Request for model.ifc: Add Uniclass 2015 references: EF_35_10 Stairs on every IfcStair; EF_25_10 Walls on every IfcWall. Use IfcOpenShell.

First a look at what the model holds.

```python
import ifcopenshell

model = ifcopenshell.open("model.ifc")
print(model.schema)
print("classifications:", [c.Name for c in model.by_type("IfcClassification")])
for ifc_class in ("IfcDoor", "IfcRoof", "IfcStair", "IfcWall", "IfcWindow"):
    print(ifc_class, len(model.by_type(ifc_class)))
```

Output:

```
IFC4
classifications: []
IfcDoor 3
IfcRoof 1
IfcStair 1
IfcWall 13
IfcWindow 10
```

```python
import ifcopenshell
import ifcopenshell.api.classification

model = ifcopenshell.open("model.ifc")

system = ifcopenshell.api.classification.add_classification(model, classification="Uniclass 2015")

codes = {
    "IfcStair": ("EF_35_10", "Stairs"),
    "IfcWall": ("EF_25_10", "Walls"),
}
for ifc_class, (code, name) in codes.items():
    products = model.by_type(ifc_class)
    ifcopenshell.api.classification.add_reference(
        model, products=products, classification=system, identification=code, name=name
    )
    print(code, len(products))

model.write("model_updated.ifc")
```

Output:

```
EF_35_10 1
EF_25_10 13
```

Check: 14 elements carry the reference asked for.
